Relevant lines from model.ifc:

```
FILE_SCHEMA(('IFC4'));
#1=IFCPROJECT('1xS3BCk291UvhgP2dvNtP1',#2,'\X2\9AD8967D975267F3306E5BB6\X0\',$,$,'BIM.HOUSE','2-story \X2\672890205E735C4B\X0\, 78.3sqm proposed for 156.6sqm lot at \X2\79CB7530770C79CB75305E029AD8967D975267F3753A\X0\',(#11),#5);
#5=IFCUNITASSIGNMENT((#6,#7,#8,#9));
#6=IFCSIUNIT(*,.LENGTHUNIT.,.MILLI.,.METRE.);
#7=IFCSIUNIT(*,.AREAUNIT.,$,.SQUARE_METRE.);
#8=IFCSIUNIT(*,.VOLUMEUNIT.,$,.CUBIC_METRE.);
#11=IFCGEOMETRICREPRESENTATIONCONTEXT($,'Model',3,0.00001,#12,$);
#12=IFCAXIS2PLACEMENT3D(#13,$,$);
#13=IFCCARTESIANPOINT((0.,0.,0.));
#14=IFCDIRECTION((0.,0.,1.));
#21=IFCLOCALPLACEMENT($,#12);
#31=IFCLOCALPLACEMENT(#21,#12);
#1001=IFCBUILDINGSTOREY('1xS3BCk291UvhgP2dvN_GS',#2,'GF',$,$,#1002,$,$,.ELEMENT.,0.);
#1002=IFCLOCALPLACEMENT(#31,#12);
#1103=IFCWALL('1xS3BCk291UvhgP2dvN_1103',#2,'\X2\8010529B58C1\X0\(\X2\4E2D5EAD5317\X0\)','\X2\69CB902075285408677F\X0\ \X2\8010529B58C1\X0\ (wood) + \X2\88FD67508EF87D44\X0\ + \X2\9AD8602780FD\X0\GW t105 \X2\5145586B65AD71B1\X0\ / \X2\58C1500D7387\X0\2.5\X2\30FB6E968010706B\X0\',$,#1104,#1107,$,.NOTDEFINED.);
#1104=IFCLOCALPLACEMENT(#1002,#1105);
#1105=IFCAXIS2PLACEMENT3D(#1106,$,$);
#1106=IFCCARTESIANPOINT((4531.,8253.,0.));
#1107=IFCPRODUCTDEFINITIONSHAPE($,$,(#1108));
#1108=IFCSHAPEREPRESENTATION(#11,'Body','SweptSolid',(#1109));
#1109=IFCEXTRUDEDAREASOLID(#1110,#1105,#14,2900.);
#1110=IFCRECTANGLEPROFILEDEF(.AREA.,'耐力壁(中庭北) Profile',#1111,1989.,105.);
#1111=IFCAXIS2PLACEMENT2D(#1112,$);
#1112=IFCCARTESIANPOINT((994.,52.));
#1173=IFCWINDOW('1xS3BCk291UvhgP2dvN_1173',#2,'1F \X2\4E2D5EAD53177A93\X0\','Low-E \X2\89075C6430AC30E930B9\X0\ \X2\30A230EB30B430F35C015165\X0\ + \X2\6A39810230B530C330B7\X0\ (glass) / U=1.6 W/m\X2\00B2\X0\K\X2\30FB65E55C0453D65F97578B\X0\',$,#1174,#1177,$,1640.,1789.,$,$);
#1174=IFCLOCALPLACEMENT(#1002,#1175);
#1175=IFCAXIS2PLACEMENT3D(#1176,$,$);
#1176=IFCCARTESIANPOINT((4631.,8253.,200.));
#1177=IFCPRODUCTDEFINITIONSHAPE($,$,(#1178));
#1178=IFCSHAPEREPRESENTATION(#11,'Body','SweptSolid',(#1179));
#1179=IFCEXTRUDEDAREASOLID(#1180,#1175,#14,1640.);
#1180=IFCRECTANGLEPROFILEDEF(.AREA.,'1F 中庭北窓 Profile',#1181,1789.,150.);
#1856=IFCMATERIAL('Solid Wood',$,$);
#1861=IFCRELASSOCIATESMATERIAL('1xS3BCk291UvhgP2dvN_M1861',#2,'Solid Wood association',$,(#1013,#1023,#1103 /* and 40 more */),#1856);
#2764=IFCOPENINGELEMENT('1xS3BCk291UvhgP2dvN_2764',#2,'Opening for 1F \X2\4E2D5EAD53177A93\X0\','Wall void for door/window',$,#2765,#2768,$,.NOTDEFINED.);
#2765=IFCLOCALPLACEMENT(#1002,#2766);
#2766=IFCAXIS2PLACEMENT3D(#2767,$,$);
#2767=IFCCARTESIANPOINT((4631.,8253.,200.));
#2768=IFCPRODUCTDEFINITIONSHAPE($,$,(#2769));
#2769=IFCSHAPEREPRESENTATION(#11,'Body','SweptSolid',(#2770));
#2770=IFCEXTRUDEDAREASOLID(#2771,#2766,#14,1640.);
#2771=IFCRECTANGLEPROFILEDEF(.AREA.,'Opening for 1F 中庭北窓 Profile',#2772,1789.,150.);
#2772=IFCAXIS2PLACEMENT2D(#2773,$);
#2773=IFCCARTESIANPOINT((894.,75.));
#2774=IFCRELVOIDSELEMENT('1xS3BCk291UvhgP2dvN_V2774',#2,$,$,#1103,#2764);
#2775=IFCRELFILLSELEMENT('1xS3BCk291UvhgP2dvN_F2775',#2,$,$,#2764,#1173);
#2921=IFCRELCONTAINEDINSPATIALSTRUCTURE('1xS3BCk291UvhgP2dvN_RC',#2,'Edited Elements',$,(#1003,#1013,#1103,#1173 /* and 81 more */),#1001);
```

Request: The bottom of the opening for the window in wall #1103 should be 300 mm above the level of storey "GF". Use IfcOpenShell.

```python
import numpy as np
import ifcopenshell
import ifcopenshell.api.geometry
import ifcopenshell.geom
import ifcopenshell.util.element
import ifcopenshell.util.placement
import ifcopenshell.util.shape
import ifcopenshell.util.unit

model = ifcopenshell.open("model.ifc")
unit_scale = ifcopenshell.util.unit.calculate_unit_scale(model)

window = model.by_id(1173)
opening = window.FillsVoids[0].RelatingOpeningElement
storey = ifcopenshell.util.element.get_container(window, ifc_class="IfcBuildingStorey")
level = ifcopenshell.util.placement.get_local_placement(storey.ObjectPlacement)[2, 3]

# The opening's origin need not be at the sill, so measure its lowest point.
shape = ifcopenshell.geom.create_shape(ifcopenshell.geom.settings(), opening)
bottom = ifcopenshell.util.shape.get_shape_bottom_elevation(shape, shape.geometry) / unit_scale
dz = level + 0.3 / unit_scale - bottom

shift = np.array([0.0, 0.0, dz])
# The window is not placed relative to its opening, so move both.
for product in (opening, window):
    matrix = ifcopenshell.util.placement.get_local_placement(product.ObjectPlacement)
    matrix[:3, 3] += shift
    ifcopenshell.api.geometry.edit_object_placement(model, product=product, matrix=matrix, is_si=False)

print(f"moved by {dz * unit_scale:+.3f} m")

model.write("model_edited.ifc")
```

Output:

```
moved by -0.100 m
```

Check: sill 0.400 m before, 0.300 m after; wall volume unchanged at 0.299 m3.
